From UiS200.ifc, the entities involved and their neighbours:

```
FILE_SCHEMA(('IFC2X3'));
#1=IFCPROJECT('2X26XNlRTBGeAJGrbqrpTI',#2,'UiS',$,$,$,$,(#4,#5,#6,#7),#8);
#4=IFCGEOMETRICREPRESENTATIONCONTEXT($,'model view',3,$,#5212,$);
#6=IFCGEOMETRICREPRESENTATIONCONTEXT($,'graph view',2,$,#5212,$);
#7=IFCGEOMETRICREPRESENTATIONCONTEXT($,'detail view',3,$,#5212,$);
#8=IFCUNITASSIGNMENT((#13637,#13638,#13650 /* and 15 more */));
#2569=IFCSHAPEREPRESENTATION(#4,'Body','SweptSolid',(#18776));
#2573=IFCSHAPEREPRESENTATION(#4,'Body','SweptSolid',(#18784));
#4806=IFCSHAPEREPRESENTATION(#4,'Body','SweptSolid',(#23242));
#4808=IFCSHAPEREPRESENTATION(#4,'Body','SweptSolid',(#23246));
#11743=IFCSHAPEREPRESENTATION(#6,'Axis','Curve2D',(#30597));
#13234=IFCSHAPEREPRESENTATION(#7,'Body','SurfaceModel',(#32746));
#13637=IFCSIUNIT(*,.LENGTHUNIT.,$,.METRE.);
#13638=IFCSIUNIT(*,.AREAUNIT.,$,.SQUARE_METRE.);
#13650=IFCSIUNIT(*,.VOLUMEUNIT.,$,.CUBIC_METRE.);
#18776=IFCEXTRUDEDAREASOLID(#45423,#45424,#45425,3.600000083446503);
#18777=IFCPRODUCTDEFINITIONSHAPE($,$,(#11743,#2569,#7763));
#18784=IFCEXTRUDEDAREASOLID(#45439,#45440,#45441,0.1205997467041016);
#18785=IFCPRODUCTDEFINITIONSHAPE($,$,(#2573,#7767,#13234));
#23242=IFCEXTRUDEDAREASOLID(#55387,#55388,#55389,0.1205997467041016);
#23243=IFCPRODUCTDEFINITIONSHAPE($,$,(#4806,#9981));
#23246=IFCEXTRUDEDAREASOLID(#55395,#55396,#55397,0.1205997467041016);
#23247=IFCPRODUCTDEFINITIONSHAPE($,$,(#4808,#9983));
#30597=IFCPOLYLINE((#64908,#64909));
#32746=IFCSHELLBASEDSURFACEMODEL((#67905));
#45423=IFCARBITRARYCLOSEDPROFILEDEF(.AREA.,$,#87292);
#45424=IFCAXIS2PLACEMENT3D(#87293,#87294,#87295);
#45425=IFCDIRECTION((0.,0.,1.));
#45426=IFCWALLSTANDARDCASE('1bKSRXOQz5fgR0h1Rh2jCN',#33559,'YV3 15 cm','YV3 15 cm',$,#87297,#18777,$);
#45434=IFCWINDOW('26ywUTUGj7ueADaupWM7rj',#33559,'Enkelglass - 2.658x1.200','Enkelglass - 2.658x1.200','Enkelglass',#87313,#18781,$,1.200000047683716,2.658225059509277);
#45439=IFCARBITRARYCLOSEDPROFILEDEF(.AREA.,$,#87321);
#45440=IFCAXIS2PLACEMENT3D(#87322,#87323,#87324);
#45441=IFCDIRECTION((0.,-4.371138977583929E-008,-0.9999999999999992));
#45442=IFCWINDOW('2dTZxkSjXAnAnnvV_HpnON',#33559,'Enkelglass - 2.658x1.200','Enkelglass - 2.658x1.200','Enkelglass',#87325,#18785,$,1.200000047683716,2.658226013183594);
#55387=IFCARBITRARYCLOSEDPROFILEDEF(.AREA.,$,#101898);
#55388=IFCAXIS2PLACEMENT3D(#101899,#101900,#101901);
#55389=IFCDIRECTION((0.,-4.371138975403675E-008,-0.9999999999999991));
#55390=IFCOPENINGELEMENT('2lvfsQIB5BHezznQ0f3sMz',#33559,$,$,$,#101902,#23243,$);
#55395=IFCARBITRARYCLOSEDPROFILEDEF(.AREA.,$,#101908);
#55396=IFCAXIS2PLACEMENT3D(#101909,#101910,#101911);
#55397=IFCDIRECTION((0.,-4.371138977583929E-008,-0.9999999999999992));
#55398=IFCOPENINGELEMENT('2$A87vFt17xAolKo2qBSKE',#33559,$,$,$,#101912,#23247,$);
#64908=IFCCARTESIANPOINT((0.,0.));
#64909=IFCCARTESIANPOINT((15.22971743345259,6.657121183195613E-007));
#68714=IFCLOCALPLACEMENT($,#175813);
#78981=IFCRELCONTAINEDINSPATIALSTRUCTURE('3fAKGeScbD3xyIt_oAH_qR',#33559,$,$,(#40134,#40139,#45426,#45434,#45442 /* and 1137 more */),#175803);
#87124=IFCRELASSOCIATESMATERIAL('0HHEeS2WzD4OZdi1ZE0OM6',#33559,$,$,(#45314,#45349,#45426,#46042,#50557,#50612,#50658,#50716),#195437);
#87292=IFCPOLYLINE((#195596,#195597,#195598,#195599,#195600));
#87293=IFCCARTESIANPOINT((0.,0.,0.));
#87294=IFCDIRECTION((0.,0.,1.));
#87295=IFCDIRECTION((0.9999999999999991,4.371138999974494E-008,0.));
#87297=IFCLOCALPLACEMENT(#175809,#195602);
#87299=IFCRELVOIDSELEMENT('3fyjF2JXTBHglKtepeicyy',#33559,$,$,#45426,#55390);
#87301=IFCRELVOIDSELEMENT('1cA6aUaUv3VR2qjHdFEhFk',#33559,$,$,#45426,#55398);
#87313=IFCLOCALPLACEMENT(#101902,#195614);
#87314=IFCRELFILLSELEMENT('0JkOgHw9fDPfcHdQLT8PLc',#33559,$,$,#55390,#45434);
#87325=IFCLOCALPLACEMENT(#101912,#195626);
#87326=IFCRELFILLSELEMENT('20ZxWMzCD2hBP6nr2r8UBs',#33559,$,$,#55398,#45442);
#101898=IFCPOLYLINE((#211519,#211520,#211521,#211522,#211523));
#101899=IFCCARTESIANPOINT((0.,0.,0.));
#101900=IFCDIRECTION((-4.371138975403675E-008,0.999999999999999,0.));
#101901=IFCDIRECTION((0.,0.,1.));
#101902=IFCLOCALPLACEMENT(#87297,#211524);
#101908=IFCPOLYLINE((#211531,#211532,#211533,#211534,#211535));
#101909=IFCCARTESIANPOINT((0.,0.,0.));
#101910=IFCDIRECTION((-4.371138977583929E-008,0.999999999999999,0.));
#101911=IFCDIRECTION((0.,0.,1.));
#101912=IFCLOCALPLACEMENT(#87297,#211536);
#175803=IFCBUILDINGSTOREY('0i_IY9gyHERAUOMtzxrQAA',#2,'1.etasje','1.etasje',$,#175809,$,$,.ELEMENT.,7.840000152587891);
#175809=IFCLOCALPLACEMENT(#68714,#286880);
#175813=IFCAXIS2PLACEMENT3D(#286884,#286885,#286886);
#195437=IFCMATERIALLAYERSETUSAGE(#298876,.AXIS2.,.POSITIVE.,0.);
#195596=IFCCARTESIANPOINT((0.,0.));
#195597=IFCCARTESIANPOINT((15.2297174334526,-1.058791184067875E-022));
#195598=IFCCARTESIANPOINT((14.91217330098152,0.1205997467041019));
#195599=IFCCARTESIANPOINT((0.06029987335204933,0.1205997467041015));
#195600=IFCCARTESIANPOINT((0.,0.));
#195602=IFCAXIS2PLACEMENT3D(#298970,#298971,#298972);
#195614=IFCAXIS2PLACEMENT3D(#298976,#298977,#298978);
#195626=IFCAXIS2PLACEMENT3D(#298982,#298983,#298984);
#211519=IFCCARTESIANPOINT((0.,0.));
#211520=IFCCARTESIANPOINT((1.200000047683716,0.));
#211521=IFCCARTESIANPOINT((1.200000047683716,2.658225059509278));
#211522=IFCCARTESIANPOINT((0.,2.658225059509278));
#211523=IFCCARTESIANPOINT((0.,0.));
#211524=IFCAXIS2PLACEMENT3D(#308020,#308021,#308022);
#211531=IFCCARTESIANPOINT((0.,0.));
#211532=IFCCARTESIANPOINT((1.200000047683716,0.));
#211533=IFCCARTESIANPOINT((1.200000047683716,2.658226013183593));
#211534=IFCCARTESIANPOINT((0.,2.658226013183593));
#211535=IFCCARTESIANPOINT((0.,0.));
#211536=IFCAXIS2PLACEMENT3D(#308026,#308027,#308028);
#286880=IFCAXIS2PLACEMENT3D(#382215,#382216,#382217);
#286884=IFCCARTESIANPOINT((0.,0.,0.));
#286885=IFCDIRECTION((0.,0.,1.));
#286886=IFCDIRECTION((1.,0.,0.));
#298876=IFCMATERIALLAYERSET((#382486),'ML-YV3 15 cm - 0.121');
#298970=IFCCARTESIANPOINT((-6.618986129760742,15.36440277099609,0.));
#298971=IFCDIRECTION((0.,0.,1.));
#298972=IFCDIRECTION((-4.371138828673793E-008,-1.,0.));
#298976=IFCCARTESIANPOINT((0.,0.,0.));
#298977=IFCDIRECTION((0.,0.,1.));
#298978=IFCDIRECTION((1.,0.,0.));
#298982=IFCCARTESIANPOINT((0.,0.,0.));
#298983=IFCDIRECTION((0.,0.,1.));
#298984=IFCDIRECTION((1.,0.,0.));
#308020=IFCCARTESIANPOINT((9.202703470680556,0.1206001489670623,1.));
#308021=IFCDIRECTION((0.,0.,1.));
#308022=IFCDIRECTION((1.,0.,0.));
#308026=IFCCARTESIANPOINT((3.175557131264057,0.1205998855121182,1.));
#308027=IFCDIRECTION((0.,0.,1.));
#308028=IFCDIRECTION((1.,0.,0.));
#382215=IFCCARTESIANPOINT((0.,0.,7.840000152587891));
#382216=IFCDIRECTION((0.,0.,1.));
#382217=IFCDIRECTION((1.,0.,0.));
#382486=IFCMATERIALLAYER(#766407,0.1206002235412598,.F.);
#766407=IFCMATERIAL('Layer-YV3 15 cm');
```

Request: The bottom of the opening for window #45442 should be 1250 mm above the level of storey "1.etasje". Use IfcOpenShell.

```python
import numpy as np
import ifcopenshell
import ifcopenshell.api.geometry
import ifcopenshell.geom
import ifcopenshell.util.element
import ifcopenshell.util.placement
import ifcopenshell.util.shape
import ifcopenshell.util.unit

model = ifcopenshell.open("UiS200.ifc")
unit_scale = ifcopenshell.util.unit.calculate_unit_scale(model)

window = model.by_id(45442)
opening = window.FillsVoids[0].RelatingOpeningElement
storey = ifcopenshell.util.element.get_container(window, ifc_class="IfcBuildingStorey")
level = ifcopenshell.util.placement.get_local_placement(storey.ObjectPlacement)[2, 3]

# The opening's origin need not be at the sill, so measure its lowest point.
shape = ifcopenshell.geom.create_shape(ifcopenshell.geom.settings(), opening)
bottom = ifcopenshell.util.shape.get_shape_bottom_elevation(shape, shape.geometry) / unit_scale
dz = level + 1.25 / unit_scale - bottom

shift = np.array([0.0, 0.0, dz])
# The window is placed relative to its opening, so it follows when the opening moves.
matrix = ifcopenshell.util.placement.get_local_placement(opening.ObjectPlacement)
matrix[:3, 3] += shift
ifcopenshell.api.geometry.edit_object_placement(
    model, product=opening, matrix=matrix, is_si=False, should_transform_children=True
)

print(f"moved by {dz * unit_scale:+.3f} m")

model.write("UiS200_updated.ifc")
```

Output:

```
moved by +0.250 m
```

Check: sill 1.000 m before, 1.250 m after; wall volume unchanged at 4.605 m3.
